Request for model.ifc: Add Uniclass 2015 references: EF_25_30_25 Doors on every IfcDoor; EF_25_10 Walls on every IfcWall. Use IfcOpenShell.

First a look at what the model holds.

```python
import ifcopenshell

model = ifcopenshell.open("model.ifc")
print(model.schema)
print("classifications:", [c.Name for c in model.by_type("IfcClassification")])
for ifc_class in ("IfcDoor", "IfcRoof", "IfcStair", "IfcWall", "IfcWindow"):
    print(ifc_class, len(model.by_type(ifc_class)))
```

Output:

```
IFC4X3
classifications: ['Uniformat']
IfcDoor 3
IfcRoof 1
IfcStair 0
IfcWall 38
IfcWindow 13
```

```python
import ifcopenshell
import ifcopenshell.api.classification

model = ifcopenshell.open("model.ifc")

system = ifcopenshell.api.classification.add_classification(model, classification="Uniclass 2015")

codes = {
    "IfcDoor": ("EF_25_30_25", "Doors"),
    "IfcWall": ("EF_25_10", "Walls"),
}
for ifc_class, (code, name) in codes.items():
    products = model.by_type(ifc_class)
    ifcopenshell.api.classification.add_reference(
        model, products=products, classification=system, identification=code, name=name
    )
    print(code, len(products))

model.write("model_updated.ifc")
```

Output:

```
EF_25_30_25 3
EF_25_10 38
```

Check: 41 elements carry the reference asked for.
